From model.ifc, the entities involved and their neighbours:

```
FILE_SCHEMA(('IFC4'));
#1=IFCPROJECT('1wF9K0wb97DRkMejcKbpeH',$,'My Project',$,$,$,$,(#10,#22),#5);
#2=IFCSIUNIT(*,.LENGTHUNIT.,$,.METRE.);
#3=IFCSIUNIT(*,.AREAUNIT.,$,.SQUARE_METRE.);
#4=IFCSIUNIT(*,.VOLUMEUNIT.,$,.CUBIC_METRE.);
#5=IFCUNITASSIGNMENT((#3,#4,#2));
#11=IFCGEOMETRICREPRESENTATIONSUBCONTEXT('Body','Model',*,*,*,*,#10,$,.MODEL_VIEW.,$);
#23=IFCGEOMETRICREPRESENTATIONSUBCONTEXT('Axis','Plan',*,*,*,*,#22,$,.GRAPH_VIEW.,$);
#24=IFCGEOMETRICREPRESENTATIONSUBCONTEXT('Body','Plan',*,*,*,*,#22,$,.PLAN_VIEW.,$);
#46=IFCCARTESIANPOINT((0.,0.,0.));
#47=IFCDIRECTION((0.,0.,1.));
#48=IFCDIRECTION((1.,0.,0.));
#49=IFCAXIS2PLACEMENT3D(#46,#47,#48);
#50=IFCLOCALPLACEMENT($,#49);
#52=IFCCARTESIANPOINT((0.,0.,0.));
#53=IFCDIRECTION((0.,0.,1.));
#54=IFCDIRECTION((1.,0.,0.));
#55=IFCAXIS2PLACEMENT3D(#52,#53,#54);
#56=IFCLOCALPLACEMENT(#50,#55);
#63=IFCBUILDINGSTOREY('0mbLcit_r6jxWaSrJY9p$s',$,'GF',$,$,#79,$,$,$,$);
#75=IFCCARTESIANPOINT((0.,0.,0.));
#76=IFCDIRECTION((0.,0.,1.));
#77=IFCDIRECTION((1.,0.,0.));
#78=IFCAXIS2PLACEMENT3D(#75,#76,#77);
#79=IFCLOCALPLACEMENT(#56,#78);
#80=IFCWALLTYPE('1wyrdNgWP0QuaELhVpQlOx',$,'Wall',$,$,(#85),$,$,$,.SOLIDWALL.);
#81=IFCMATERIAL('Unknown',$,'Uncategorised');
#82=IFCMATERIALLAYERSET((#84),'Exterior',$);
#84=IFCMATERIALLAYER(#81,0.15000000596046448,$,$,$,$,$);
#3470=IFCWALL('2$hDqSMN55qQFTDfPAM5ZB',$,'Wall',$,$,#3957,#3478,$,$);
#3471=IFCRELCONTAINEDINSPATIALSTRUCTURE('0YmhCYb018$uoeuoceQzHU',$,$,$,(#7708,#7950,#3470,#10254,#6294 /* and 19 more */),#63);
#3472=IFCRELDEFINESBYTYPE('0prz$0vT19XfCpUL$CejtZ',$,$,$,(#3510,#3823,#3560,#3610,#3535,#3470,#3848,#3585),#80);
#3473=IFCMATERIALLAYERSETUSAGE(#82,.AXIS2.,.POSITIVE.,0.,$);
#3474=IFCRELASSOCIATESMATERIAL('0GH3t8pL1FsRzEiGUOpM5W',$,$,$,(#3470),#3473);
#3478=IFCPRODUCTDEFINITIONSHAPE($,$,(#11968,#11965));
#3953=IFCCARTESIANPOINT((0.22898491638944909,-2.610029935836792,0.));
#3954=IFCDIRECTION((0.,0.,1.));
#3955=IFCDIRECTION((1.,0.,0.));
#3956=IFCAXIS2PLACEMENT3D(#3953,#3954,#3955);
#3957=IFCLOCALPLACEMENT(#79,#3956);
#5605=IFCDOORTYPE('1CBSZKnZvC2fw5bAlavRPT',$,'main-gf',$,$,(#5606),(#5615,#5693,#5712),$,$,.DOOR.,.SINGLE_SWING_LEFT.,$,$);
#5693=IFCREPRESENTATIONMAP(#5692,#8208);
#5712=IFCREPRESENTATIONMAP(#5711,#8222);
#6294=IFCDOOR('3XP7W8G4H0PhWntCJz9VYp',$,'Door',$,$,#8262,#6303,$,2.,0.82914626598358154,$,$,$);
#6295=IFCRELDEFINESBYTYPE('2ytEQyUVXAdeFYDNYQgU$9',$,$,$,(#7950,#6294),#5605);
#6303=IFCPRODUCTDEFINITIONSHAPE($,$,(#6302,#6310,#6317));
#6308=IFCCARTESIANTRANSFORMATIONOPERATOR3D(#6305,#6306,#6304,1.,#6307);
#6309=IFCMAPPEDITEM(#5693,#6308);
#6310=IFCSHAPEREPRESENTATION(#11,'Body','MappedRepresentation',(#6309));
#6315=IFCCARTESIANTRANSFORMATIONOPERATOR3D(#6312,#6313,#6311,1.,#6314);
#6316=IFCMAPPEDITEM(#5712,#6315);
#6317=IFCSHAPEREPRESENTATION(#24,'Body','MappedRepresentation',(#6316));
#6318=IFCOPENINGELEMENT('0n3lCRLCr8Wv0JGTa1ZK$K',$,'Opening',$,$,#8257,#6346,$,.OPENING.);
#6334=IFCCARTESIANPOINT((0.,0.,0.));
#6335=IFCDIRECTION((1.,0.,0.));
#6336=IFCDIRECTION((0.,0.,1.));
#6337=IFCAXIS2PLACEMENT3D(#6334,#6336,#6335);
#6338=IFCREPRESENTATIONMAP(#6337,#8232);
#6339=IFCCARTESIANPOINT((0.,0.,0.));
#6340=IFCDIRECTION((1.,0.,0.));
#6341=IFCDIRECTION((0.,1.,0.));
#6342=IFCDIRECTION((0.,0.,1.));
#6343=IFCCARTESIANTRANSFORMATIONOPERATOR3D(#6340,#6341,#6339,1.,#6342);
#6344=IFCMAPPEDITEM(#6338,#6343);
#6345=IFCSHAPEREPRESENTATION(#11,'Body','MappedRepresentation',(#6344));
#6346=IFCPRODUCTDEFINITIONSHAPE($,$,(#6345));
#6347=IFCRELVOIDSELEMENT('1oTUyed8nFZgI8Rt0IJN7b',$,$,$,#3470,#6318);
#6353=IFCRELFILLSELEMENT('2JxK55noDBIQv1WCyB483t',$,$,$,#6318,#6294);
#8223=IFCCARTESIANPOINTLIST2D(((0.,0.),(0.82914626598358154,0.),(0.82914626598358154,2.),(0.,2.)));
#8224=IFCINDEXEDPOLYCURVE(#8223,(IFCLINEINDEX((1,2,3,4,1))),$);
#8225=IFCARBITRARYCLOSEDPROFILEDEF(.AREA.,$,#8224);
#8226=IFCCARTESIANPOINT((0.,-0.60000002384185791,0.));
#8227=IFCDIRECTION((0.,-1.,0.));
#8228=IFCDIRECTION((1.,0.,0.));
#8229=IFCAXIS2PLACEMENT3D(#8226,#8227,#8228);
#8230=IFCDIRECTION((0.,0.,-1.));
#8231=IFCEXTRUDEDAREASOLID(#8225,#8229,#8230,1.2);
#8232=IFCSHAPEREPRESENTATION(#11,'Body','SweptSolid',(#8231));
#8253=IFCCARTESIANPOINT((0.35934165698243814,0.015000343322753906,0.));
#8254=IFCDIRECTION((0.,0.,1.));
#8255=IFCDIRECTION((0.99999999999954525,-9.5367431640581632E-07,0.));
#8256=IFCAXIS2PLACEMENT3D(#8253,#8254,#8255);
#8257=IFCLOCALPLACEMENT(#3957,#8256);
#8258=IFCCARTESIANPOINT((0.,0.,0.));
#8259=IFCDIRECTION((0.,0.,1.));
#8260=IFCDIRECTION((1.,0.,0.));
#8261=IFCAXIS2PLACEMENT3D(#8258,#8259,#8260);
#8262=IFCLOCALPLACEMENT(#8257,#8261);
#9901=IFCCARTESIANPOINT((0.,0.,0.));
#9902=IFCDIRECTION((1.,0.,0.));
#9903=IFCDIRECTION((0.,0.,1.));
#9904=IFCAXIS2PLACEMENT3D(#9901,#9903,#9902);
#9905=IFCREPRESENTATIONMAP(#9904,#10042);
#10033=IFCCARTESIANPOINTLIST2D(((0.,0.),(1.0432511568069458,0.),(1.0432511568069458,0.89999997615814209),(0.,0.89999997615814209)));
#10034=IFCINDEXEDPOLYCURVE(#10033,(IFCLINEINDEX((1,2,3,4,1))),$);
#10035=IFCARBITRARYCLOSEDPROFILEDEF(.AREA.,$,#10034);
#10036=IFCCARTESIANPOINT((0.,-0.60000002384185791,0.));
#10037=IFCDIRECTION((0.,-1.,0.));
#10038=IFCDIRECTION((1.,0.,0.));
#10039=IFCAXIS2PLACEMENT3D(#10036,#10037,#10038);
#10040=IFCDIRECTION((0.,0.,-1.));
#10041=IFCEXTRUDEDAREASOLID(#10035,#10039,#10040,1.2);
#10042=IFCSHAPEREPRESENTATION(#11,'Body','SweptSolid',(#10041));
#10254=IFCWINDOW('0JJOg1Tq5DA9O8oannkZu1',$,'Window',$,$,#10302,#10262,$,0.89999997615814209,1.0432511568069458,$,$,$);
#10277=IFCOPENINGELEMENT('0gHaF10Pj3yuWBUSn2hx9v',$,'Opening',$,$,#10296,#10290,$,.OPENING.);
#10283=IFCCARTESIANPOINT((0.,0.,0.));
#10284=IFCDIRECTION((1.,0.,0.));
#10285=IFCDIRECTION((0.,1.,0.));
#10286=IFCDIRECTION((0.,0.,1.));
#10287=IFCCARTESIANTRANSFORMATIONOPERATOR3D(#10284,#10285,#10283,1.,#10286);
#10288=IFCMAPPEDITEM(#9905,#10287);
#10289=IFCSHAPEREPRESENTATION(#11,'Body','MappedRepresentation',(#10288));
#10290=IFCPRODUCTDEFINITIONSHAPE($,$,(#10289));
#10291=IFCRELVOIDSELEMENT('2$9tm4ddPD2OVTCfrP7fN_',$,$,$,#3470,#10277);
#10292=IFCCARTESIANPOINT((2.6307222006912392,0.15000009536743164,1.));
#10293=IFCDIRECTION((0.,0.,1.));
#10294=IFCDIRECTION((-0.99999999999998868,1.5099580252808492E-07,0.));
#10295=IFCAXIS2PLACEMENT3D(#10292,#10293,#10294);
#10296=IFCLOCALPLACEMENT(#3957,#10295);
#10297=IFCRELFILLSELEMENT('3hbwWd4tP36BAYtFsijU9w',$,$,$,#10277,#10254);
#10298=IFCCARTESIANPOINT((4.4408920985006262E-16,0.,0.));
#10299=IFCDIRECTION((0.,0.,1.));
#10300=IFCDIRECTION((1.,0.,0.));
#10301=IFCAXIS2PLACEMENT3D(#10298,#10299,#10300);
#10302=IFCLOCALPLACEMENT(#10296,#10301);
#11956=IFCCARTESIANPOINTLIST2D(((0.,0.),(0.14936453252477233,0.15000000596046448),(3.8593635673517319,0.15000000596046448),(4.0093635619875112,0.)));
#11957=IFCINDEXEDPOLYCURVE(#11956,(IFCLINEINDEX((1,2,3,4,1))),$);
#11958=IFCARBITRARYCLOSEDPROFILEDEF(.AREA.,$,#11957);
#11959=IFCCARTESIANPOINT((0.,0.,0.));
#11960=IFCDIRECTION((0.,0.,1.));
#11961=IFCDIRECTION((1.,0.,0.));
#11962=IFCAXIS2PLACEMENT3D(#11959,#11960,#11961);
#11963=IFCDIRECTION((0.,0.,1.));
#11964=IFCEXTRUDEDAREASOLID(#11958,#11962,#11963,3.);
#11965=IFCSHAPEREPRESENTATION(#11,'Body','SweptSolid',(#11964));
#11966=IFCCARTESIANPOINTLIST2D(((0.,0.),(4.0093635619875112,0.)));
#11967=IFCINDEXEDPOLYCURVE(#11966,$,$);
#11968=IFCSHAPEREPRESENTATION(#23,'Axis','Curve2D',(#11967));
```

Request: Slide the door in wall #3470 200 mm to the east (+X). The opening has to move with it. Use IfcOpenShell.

```python
import ifcopenshell
import ifcopenshell.api.geometry
import ifcopenshell.util.placement

model = ifcopenshell.open("model.ifc")

door = model.by_id(6294)
opening = door.FillsVoids[0].RelatingOpeningElement
wall = opening.VoidsElements[0].RelatingBuildingElement

wall_matrix = ifcopenshell.util.placement.get_local_placement(wall.ObjectPlacement)
shift = wall_matrix[:3, 0] * 0.2
before = ifcopenshell.util.placement.get_local_placement(door.ObjectPlacement)[:3, 3].copy()

# The door is placed relative to its opening, so it follows when the opening moves.
matrix = ifcopenshell.util.placement.get_local_placement(opening.ObjectPlacement)
matrix[:3, 3] += shift
ifcopenshell.api.geometry.edit_object_placement(
    model, product=opening, matrix=matrix, is_si=False, should_transform_children=True
)

after = ifcopenshell.util.placement.get_local_placement(door.ObjectPlacement)[:3, 3]
print("door moved by", (after - before).round(3) + 0.0)

model.write("model_rev.ifc")
```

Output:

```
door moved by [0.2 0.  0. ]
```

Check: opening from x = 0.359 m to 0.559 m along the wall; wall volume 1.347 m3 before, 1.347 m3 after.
